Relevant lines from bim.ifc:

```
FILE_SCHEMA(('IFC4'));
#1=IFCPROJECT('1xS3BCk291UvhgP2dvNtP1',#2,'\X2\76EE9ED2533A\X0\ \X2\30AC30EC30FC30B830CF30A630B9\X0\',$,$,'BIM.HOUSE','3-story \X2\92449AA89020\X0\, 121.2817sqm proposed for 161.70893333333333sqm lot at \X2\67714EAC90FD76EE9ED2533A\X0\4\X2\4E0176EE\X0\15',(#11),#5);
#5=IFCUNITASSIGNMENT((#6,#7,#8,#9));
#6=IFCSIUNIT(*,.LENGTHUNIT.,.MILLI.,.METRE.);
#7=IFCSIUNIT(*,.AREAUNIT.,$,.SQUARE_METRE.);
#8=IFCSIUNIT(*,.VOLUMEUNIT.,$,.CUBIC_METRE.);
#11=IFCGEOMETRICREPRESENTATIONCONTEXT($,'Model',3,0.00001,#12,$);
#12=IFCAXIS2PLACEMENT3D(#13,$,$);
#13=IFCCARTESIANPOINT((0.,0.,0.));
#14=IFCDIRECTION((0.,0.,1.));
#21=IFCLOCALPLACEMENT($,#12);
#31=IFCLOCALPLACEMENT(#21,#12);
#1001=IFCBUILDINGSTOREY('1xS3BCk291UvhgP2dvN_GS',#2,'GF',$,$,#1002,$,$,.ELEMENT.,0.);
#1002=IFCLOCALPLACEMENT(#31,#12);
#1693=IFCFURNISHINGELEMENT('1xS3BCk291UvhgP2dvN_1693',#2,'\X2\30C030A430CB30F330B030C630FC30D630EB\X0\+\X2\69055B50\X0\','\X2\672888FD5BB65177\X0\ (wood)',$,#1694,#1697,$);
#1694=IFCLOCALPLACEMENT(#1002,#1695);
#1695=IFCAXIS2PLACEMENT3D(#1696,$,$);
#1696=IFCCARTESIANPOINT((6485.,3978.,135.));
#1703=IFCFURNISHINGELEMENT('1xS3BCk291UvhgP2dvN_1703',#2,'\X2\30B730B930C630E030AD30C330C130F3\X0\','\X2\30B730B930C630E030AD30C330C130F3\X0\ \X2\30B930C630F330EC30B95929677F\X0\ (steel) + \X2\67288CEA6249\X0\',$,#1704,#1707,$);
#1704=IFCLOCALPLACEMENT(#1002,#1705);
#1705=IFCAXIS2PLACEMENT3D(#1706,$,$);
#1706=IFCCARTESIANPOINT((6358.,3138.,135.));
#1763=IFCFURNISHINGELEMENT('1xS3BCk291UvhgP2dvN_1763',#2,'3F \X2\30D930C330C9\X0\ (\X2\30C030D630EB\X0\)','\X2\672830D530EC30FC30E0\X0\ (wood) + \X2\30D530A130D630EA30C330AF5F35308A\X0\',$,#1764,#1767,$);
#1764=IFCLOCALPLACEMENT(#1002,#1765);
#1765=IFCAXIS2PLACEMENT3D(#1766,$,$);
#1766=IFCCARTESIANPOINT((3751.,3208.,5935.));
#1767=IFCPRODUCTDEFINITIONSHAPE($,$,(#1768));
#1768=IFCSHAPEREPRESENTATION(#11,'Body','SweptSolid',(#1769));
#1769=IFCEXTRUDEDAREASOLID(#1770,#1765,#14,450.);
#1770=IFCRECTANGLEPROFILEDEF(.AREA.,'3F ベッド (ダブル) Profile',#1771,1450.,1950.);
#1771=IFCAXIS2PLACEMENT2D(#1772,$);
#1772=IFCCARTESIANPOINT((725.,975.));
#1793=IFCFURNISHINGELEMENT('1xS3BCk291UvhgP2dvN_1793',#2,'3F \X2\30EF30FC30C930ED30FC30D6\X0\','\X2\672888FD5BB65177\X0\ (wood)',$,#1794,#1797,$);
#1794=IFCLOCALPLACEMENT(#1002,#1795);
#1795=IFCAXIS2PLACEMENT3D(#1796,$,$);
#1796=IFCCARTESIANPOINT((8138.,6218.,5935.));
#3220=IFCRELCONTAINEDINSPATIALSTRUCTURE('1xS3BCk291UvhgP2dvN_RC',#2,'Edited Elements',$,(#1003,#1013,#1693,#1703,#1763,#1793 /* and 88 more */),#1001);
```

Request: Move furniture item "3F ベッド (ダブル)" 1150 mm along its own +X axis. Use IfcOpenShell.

```python
import ifcopenshell
import ifcopenshell.api.geometry
import ifcopenshell.util.placement
import ifcopenshell.util.unit

model = ifcopenshell.open("bim.ifc")
unit_scale = ifcopenshell.util.unit.calculate_unit_scale(model)

item = model.by_id(1763)
matrix = ifcopenshell.util.placement.get_local_placement(item.ObjectPlacement)
matrix[:3, 3] += matrix[:3, 0] * 1.15 / unit_scale
ifcopenshell.api.geometry.edit_object_placement(model, product=item, matrix=matrix, is_si=False)

print(ifcopenshell.util.placement.get_local_placement(item.ObjectPlacement).round(3) + 0.0)

model.write("bim_v2.ifc")
```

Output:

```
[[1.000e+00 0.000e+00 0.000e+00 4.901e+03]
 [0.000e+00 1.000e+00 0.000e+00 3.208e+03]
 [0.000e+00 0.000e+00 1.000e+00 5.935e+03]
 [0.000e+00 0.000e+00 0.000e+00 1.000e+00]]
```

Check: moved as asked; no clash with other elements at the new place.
